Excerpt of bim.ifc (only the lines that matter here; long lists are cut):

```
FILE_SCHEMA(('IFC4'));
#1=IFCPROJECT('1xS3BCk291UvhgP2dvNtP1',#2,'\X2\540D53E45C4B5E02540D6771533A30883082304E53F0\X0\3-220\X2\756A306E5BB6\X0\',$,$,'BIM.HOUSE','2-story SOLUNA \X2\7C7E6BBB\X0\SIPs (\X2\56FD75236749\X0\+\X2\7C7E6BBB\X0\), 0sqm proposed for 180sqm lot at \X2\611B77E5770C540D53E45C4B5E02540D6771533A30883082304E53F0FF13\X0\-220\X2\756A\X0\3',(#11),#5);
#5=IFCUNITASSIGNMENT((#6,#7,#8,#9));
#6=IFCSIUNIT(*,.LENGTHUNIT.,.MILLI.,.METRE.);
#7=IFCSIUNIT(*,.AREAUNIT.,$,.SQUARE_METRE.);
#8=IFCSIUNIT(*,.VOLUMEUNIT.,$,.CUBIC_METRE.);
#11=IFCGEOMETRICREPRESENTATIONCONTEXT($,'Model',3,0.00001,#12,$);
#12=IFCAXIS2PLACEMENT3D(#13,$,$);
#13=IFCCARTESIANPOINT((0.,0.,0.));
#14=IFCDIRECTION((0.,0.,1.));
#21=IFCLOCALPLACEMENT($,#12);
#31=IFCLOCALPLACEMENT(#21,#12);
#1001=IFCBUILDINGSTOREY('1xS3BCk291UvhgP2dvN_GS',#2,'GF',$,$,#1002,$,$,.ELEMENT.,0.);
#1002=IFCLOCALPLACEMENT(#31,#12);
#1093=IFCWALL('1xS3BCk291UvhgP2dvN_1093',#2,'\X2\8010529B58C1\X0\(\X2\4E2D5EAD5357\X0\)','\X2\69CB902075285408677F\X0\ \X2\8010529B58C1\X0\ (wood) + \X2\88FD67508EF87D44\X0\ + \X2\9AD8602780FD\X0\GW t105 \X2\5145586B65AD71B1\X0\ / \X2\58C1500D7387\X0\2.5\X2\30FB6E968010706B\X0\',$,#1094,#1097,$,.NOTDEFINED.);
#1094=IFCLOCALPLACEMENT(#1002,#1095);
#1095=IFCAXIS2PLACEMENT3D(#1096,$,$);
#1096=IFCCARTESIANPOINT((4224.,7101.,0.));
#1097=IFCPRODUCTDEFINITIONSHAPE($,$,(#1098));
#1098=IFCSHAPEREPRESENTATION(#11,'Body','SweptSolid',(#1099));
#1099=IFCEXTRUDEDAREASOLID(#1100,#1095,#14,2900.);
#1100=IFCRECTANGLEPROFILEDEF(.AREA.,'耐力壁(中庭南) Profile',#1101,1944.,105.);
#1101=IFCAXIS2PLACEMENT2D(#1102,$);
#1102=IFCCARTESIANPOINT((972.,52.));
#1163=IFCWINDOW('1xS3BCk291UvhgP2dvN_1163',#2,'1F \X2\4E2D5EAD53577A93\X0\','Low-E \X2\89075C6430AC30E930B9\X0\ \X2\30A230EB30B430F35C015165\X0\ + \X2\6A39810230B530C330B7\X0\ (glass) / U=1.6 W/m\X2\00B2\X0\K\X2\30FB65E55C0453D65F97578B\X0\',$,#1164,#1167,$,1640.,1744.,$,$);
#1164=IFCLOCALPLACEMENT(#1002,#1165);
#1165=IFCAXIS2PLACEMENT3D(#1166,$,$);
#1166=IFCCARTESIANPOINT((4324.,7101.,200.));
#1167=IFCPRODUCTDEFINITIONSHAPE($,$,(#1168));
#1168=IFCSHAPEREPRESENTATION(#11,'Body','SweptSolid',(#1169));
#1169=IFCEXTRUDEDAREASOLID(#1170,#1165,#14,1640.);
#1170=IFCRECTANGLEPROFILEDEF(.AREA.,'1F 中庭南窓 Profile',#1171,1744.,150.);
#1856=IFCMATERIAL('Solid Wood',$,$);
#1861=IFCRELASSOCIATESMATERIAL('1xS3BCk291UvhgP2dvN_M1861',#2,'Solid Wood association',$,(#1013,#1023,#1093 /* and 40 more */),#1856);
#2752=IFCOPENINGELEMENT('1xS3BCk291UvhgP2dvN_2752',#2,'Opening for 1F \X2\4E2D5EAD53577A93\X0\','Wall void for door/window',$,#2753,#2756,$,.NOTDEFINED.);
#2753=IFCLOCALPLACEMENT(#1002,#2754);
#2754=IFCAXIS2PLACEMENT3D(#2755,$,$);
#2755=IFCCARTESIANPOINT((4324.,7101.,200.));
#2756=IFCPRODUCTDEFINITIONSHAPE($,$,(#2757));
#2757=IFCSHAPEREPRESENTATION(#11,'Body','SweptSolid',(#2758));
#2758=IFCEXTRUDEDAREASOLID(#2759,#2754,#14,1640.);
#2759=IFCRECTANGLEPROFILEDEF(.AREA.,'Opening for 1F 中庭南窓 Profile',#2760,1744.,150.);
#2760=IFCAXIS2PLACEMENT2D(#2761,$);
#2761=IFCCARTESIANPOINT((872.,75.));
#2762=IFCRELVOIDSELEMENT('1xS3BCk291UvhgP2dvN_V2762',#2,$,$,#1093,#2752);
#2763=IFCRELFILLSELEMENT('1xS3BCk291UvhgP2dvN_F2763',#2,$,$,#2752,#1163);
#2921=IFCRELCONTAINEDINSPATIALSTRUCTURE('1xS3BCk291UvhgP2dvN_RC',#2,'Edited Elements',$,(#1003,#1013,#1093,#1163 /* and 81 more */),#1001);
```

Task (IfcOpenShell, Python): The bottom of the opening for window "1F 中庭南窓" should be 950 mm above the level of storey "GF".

```python
import numpy as np
import ifcopenshell
import ifcopenshell.api.geometry
import ifcopenshell.geom
import ifcopenshell.util.element
import ifcopenshell.util.placement
import ifcopenshell.util.shape
import ifcopenshell.util.unit

model = ifcopenshell.open("bim.ifc")
unit_scale = ifcopenshell.util.unit.calculate_unit_scale(model)

window = model.by_guid("1xS3BCk291UvhgP2dvN_1163")
opening = window.FillsVoids[0].RelatingOpeningElement
storey = ifcopenshell.util.element.get_container(window, ifc_class="IfcBuildingStorey")
level = ifcopenshell.util.placement.get_local_placement(storey.ObjectPlacement)[2, 3]

# The opening's origin need not be at the sill, so measure its lowest point.
shape = ifcopenshell.geom.create_shape(ifcopenshell.geom.settings(), opening)
bottom = ifcopenshell.util.shape.get_shape_bottom_elevation(shape, shape.geometry) / unit_scale
dz = level + 950.0 - bottom

shift = np.array([0.0, 0.0, dz])
# The window is not placed relative to its opening, so move both.
for product in (opening, window):
    matrix = ifcopenshell.util.placement.get_local_placement(product.ObjectPlacement)
    matrix[:3, 3] += shift
    ifcopenshell.api.geometry.edit_object_placement(model, product=product, matrix=matrix, is_si=False)

print(f"moved by {dz * unit_scale:+.3f} m")

model.write("bim_updated.ifc")
```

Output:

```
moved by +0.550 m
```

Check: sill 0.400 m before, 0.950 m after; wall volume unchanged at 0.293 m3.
